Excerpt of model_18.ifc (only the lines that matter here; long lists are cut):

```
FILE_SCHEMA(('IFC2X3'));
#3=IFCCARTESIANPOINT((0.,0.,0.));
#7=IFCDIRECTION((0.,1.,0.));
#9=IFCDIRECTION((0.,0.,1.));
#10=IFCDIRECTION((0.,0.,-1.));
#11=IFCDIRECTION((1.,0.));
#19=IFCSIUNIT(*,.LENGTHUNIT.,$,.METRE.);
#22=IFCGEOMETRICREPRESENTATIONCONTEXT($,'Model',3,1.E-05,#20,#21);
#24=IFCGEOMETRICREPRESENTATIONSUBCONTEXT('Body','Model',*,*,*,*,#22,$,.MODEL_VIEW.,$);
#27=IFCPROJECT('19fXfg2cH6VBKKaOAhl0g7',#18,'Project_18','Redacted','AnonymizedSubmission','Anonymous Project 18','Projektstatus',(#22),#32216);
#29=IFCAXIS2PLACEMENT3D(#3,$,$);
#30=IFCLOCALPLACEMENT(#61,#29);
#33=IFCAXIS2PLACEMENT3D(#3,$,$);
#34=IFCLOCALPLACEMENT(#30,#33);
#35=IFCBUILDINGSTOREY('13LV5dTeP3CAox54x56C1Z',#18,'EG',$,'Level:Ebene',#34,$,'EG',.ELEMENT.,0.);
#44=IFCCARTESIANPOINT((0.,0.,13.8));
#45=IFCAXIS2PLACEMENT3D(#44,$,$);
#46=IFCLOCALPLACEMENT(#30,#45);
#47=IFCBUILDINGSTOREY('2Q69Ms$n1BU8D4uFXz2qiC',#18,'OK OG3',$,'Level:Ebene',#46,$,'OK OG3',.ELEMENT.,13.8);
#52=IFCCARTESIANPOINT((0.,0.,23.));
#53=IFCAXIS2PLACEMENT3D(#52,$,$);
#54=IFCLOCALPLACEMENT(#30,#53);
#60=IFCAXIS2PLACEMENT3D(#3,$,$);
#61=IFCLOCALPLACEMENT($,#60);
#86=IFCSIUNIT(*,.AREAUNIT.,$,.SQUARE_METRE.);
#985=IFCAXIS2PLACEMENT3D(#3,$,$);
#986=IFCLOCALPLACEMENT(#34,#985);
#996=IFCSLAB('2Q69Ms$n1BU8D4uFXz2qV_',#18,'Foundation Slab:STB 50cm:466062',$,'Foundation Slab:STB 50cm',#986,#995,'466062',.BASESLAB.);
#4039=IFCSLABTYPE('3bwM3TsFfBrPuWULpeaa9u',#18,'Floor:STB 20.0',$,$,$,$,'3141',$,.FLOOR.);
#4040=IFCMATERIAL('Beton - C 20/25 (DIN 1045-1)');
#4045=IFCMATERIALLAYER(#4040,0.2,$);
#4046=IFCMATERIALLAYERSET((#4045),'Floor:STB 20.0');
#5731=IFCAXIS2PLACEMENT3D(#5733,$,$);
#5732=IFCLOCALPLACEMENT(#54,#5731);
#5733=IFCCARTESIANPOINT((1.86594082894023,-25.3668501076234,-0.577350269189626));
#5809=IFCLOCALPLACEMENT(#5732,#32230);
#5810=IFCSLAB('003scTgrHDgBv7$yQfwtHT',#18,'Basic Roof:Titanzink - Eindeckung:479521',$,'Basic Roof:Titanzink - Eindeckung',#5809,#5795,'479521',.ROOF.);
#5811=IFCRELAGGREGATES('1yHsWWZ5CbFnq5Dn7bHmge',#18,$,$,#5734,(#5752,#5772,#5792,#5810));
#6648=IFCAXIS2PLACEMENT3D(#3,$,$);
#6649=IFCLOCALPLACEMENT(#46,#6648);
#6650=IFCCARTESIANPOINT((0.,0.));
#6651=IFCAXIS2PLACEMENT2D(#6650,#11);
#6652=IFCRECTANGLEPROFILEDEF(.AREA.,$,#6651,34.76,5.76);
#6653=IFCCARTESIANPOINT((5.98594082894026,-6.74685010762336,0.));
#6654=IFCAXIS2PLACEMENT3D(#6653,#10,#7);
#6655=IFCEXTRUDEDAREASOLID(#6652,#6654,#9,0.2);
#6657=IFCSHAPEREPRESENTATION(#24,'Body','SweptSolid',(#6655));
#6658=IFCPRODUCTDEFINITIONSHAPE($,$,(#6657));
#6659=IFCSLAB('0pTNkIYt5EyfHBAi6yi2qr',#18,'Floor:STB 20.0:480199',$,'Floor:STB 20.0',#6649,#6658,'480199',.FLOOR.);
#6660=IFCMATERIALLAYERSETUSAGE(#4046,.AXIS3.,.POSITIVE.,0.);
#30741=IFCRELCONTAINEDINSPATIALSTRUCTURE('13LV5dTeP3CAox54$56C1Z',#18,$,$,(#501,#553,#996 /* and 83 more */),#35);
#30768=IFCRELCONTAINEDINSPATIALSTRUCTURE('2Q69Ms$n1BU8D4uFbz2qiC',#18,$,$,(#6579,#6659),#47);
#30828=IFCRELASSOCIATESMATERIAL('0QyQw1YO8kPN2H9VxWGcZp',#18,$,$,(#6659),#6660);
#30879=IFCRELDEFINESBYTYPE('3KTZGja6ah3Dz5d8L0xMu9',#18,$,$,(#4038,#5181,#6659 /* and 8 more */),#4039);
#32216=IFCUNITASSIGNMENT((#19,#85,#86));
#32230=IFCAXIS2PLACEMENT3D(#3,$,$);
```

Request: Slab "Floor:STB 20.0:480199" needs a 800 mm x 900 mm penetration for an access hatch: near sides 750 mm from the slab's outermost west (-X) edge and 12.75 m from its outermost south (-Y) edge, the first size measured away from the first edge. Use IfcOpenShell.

```python
import numpy as np
import ifcopenshell
import ifcopenshell.api.feature
import ifcopenshell.api.geometry
import ifcopenshell.api.root
import ifcopenshell.geom
import ifcopenshell.util.placement
import ifcopenshell.util.representation
import ifcopenshell.util.shape
import ifcopenshell.util.unit

model = ifcopenshell.open("model_18.ifc")
unit_scale = ifcopenshell.util.unit.calculate_unit_scale(model)
settings = ifcopenshell.geom.settings()


def volume(element):
    """Net volume in cubic metres, openings subtracted."""
    shape = ifcopenshell.geom.create_shape(settings, element)
    return ifcopenshell.util.shape.get_volume(shape.geometry)


slab = model.by_guid("0pTNkIYt5EyfHBAi6yi2qr")
before = volume(slab)

# Extent in the slab's own axes, in metres. The edges named are its -X and -Y sides.
slab_shape = ifcopenshell.geom.create_shape(settings, slab)
vertices = ifcopenshell.util.shape.get_vertices(slab_shape.geometry)
x_min, y_min, bottom = vertices.min(axis=0)
top = vertices[:, 2].max()

opening = ifcopenshell.api.root.create_entity(model, ifc_class="IfcOpeningElement", name="Access hatch opening")
context = ifcopenshell.util.representation.get_context(model, "Model", "Body", "MODEL_VIEW")
width, depth = 0.8, 0.9
outline = [(0.0, 0.0), (width, 0.0), (width, depth), (0.0, depth), (0.0, 0.0)]
# Overshoot both faces by 50 mm so the cut is clean.
shape = ifcopenshell.api.geometry.add_slab_representation(
    model, context=context, depth=top - bottom + 0.1, polyline=outline
)
ifcopenshell.api.geometry.assign_representation(model, product=opening, representation=shape)

matrix = ifcopenshell.util.placement.get_local_placement(slab.ObjectPlacement)
matrix[:, 3] = matrix @ np.append(np.array([x_min + 0.75, y_min + 12.75, bottom - 0.05]) / unit_scale, 1.0)
ifcopenshell.api.geometry.edit_object_placement(model, product=opening, matrix=matrix, is_si=False)
ifcopenshell.api.feature.add_feature(model, feature=opening, element=slab)

after = volume(slab)

print(f"slab volume {before:.3f} -> {after:.3f} m3")

model.write("model_18_rev.ifc")
```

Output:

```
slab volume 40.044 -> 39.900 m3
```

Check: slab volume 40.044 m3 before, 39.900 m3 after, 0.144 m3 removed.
